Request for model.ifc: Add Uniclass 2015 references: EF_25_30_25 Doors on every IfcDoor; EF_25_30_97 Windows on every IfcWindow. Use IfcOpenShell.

First a look at what the model holds.

```python
import ifcopenshell

model = ifcopenshell.open("model.ifc")
print(model.schema)
print("classifications:", [c.Name for c in model.by_type("IfcClassification")])
for ifc_class in ("IfcDoor", "IfcRoof", "IfcStair", "IfcWall", "IfcWindow"):
    print(ifc_class, len(model.by_type(ifc_class)))
```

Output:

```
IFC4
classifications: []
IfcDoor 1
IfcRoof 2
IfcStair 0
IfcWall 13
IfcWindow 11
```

```python
import ifcopenshell
import ifcopenshell.api.classification

model = ifcopenshell.open("model.ifc")

system = ifcopenshell.api.classification.add_classification(model, classification="Uniclass 2015")

codes = {
    "IfcDoor": ("EF_25_30_25", "Doors"),
    "IfcWindow": ("EF_25_30_97", "Windows"),
}
for ifc_class, (code, name) in codes.items():
    products = model.by_type(ifc_class)
    ifcopenshell.api.classification.add_reference(
        model, products=products, classification=system, identification=code, name=name
    )
    print(code, len(products))

model.write("model_v2.ifc")
```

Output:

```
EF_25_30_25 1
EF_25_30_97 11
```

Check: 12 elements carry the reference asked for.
